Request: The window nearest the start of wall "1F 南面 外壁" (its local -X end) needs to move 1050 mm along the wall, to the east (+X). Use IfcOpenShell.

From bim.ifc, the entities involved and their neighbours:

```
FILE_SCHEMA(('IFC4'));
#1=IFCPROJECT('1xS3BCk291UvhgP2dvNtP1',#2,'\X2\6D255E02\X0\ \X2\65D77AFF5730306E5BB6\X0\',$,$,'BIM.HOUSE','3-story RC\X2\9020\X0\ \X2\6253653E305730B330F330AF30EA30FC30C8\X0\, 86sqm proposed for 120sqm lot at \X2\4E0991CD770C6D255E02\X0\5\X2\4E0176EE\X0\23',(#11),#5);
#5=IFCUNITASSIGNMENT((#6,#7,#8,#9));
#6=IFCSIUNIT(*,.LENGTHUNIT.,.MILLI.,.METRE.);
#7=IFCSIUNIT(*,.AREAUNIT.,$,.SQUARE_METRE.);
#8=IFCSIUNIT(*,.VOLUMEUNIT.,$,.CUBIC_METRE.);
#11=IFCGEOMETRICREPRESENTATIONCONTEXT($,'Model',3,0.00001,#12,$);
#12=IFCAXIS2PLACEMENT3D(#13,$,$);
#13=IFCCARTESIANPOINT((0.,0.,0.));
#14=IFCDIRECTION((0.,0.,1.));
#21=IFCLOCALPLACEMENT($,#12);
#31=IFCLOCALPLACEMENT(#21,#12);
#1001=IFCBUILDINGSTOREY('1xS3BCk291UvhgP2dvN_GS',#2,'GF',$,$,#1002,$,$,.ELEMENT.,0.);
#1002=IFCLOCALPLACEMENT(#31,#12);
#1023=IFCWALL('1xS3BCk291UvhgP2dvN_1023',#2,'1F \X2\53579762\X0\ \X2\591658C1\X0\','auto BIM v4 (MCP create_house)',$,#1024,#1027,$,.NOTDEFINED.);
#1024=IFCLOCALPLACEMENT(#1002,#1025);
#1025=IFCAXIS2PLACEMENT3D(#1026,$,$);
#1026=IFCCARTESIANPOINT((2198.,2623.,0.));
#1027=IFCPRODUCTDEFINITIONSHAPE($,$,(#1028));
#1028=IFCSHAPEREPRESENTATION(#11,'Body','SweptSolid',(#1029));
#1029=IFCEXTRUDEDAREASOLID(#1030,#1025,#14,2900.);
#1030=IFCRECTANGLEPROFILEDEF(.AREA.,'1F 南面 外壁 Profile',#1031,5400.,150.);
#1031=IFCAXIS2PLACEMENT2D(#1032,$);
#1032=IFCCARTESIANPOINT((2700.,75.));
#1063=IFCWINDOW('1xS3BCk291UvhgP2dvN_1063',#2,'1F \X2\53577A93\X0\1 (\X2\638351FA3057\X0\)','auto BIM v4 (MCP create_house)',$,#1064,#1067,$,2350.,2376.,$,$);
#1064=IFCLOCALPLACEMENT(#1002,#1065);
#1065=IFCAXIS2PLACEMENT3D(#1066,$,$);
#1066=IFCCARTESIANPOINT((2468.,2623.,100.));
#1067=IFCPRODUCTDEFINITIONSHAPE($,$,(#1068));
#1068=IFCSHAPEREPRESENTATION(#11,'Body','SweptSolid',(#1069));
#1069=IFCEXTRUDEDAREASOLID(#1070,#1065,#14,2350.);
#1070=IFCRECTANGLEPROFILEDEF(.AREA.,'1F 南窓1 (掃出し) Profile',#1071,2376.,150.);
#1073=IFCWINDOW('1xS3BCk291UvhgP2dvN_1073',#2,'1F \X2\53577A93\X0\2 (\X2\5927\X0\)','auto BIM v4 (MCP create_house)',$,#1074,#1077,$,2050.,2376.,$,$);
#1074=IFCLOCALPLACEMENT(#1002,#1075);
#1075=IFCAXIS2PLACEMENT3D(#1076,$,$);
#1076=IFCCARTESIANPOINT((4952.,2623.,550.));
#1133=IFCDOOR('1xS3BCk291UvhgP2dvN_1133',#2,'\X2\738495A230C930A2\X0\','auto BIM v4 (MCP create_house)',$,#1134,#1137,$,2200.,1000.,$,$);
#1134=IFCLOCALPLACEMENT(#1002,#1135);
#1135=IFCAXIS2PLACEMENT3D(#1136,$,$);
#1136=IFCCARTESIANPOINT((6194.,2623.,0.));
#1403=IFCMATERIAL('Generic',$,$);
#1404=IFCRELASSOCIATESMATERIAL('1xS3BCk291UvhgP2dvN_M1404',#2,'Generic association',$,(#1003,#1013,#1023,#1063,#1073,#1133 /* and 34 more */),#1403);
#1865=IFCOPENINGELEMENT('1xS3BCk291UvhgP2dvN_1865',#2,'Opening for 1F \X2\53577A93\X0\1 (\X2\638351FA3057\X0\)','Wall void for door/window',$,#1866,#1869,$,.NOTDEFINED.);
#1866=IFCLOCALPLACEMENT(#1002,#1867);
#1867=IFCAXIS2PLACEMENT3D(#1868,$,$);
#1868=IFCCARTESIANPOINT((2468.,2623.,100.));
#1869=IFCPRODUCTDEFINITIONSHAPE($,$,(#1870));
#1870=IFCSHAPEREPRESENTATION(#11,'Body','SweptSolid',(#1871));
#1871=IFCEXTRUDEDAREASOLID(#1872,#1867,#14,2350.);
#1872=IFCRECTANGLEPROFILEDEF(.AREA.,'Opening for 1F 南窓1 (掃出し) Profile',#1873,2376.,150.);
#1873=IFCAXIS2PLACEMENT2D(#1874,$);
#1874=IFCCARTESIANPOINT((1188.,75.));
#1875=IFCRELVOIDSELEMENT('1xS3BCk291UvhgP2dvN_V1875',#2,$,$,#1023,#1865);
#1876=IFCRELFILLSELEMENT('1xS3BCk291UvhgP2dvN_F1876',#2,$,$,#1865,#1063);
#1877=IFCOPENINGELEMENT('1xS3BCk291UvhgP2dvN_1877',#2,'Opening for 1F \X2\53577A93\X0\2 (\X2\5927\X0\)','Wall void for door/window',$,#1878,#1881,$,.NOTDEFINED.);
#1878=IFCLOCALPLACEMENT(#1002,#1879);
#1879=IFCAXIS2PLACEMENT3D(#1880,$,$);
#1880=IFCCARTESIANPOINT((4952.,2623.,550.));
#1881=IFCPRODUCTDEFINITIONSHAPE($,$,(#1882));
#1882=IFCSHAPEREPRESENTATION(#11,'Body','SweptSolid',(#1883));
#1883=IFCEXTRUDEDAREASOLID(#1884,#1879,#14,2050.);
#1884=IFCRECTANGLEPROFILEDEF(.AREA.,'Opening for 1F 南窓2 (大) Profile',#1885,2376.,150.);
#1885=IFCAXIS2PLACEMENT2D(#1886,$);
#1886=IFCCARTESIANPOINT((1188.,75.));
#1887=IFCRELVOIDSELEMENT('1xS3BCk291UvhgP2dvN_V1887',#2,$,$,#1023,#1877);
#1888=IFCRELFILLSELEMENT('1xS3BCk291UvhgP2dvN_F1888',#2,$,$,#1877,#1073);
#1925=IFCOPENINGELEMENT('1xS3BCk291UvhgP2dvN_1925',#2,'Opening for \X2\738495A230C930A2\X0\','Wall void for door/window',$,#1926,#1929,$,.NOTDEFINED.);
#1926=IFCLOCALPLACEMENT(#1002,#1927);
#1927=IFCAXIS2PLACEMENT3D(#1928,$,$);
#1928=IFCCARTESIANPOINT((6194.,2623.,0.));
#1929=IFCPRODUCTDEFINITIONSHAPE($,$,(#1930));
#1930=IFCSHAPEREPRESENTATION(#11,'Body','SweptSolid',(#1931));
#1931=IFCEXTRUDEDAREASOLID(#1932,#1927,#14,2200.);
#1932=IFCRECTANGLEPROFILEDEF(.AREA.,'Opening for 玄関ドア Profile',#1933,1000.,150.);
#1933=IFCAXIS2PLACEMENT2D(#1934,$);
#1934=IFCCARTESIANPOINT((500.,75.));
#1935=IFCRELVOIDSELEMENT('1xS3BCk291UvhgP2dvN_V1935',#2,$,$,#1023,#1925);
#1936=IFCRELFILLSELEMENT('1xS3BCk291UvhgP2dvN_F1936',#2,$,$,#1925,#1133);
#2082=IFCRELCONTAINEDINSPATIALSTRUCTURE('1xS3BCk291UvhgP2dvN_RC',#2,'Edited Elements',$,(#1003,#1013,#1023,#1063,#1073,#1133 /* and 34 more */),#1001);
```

```python
import ifcopenshell
import ifcopenshell.api.geometry
import ifcopenshell.util.placement

model = ifcopenshell.open("bim.ifc")

window = model.by_guid("1xS3BCk291UvhgP2dvN_1063")
opening = window.FillsVoids[0].RelatingOpeningElement
wall = opening.VoidsElements[0].RelatingBuildingElement

wall_matrix = ifcopenshell.util.placement.get_local_placement(wall.ObjectPlacement)
shift = wall_matrix[:3, 0] * 1050.0
before = ifcopenshell.util.placement.get_local_placement(window.ObjectPlacement)[:3, 3].copy()

# The window is not placed relative to its opening, so move both.
for product in (opening, window):
    matrix = ifcopenshell.util.placement.get_local_placement(product.ObjectPlacement)
    matrix[:3, 3] += shift
    ifcopenshell.api.geometry.edit_object_placement(model, product=product, matrix=matrix, is_si=False)

after = ifcopenshell.util.placement.get_local_placement(window.ObjectPlacement)[:3, 3]
print("window moved by", (after - before).round(3) + 0.0)

model.write("bim_v2.ifc")
```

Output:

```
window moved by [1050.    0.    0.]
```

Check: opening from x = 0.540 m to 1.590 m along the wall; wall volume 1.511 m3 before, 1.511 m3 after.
